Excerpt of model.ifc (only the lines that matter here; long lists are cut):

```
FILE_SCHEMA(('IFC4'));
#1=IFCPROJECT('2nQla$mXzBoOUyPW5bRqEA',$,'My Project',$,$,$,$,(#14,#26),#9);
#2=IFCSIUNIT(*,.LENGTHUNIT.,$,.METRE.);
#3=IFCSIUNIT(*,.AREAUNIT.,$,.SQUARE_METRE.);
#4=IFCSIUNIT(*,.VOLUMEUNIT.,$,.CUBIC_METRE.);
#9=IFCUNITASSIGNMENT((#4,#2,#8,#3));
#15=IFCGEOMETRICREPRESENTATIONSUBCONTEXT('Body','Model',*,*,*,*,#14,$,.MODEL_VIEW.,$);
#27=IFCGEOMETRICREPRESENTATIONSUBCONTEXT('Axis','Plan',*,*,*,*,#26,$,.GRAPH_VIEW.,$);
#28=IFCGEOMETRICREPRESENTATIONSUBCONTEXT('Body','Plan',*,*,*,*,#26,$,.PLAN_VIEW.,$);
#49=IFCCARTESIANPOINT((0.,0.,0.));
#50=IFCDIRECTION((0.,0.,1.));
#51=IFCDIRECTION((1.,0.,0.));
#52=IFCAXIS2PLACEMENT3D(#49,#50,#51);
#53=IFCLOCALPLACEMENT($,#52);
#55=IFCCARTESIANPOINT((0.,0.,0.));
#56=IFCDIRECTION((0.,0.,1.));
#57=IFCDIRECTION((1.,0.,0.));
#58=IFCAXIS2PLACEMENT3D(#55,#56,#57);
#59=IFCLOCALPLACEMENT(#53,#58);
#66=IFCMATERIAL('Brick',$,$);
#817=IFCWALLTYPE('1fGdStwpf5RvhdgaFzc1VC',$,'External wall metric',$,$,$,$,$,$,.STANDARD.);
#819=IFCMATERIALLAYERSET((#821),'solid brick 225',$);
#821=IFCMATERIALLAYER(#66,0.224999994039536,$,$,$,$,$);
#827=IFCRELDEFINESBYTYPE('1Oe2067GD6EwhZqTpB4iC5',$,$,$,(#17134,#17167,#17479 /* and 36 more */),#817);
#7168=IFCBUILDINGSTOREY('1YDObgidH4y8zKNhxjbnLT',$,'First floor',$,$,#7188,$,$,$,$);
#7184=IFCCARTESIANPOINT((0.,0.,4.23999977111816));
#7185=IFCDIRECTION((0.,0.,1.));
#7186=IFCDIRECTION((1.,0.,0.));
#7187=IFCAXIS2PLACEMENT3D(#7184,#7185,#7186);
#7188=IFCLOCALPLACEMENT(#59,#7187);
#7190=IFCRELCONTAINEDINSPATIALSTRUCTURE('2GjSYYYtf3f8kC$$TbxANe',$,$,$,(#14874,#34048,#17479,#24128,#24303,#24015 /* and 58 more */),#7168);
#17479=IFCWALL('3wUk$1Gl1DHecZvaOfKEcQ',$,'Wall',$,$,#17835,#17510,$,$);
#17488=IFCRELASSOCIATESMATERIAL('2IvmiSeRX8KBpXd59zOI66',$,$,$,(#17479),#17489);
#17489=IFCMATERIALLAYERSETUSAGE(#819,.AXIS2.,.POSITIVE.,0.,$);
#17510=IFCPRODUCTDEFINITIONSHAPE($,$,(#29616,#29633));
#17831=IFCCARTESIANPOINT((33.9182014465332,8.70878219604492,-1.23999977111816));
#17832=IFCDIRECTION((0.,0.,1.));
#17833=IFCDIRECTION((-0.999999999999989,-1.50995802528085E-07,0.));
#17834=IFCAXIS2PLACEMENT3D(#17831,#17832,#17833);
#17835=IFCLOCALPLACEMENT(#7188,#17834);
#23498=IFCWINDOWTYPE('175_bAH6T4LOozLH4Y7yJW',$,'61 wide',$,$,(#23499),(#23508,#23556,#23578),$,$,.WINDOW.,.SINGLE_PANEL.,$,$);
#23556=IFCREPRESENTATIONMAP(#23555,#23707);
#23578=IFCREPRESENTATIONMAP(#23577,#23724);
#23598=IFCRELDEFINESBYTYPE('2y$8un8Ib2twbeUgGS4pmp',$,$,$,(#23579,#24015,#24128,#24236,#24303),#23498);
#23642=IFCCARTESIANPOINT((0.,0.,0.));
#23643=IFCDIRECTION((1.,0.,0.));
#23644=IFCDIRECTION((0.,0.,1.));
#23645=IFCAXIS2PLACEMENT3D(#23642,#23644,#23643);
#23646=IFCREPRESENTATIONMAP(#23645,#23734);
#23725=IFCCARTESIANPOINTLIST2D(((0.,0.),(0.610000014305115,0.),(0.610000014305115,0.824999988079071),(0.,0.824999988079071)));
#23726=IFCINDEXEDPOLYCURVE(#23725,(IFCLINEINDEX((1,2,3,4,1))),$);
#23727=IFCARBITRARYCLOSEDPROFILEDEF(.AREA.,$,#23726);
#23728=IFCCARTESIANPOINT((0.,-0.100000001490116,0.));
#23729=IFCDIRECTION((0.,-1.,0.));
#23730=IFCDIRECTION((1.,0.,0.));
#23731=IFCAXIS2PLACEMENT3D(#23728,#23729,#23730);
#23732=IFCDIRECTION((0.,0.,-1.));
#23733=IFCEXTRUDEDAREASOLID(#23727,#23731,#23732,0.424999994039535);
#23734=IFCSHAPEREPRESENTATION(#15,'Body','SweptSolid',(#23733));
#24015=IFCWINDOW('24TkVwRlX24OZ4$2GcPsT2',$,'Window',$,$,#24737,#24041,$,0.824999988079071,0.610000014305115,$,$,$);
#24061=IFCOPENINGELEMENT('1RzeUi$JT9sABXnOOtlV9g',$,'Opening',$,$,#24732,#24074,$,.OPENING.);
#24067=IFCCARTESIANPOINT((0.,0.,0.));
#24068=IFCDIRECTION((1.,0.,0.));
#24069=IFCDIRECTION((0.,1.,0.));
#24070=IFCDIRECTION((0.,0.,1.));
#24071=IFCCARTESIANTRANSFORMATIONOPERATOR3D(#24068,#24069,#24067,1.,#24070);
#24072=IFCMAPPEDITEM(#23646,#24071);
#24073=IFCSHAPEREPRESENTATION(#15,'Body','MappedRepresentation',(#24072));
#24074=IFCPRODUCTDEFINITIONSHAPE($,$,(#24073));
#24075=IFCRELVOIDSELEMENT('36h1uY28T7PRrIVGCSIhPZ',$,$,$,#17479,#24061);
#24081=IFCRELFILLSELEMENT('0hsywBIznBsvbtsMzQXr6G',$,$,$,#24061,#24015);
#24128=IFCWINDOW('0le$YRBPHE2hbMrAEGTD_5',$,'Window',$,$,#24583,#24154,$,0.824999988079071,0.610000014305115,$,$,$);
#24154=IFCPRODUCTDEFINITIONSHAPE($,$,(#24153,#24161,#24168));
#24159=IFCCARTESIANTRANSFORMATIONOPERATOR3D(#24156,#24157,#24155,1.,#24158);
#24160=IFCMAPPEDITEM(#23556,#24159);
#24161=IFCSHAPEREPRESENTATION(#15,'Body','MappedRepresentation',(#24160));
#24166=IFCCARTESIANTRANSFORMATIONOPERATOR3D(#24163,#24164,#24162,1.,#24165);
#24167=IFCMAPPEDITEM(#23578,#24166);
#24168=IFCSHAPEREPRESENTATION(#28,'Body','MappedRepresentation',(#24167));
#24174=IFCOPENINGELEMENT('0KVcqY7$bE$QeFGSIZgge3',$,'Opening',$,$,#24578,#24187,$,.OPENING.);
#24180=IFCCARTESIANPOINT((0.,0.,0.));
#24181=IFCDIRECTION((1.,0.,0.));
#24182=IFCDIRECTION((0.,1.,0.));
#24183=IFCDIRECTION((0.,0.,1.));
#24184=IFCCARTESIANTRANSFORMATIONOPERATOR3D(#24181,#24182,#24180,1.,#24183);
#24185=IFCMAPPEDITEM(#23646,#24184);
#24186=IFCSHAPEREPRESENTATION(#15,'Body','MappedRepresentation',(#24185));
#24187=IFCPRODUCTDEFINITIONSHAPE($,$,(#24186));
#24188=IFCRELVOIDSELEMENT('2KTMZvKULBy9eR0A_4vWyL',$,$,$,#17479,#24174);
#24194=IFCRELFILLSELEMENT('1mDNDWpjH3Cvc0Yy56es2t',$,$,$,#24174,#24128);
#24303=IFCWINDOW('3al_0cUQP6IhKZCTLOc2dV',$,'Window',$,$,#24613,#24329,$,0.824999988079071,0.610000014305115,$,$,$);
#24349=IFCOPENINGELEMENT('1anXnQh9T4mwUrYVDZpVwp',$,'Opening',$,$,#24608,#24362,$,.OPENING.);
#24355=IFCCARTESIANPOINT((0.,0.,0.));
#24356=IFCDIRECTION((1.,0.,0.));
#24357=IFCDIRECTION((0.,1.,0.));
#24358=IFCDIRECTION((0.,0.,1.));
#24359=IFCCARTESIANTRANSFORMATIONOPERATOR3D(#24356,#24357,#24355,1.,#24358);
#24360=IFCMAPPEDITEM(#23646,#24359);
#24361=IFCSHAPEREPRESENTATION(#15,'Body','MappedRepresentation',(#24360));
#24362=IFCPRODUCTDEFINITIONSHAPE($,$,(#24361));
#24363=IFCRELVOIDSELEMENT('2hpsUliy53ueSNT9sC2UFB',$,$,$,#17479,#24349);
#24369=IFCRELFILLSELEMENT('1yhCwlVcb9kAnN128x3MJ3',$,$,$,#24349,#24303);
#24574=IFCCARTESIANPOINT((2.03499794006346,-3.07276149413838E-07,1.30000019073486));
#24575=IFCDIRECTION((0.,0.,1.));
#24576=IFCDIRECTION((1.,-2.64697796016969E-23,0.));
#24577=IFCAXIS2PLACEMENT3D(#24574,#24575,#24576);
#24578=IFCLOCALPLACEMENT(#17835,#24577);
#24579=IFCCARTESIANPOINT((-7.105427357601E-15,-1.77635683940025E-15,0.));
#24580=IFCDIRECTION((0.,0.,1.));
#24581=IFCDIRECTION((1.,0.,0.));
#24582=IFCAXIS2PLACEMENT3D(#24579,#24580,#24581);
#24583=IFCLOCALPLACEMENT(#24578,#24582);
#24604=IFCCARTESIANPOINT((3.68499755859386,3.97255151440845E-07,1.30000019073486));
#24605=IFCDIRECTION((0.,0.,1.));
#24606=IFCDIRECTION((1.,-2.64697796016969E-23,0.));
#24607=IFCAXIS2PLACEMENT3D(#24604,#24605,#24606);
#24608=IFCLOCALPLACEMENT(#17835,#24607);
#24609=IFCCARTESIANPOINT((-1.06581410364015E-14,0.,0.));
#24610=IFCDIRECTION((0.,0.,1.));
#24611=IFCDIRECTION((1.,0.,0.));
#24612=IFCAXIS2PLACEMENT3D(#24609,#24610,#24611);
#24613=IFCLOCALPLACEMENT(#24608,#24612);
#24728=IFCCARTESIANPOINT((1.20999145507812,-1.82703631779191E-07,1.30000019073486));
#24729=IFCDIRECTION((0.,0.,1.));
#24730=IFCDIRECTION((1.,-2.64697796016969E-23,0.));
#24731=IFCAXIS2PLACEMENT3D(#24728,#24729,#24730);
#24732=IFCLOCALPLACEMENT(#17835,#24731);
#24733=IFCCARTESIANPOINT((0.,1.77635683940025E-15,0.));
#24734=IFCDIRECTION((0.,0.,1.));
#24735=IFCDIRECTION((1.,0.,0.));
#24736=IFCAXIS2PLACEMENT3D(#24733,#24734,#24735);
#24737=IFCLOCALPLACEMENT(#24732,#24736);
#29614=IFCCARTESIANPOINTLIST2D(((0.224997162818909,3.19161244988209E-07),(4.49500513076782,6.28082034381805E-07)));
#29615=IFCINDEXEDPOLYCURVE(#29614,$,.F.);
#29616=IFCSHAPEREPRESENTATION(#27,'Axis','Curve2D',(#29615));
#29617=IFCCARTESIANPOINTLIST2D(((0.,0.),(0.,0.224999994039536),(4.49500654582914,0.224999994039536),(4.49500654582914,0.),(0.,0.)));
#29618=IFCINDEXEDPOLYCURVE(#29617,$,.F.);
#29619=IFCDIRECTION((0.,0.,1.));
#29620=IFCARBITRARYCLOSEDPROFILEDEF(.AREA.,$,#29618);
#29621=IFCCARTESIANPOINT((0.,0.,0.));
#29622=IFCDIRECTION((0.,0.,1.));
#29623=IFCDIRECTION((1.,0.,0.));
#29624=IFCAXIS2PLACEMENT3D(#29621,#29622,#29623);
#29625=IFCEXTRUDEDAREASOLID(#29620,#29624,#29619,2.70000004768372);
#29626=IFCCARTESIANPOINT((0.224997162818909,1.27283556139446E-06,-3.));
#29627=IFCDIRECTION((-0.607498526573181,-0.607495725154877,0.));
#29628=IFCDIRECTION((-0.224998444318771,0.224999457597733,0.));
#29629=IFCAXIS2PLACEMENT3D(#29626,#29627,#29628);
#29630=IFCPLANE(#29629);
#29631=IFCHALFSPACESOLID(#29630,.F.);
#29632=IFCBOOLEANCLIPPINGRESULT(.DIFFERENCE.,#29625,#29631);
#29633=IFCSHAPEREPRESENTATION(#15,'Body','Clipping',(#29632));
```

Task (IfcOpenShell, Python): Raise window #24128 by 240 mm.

```python
import numpy as np
import ifcopenshell
import ifcopenshell.api.geometry
import ifcopenshell.util.placement
import ifcopenshell.util.unit

model = ifcopenshell.open("model.ifc")
unit_scale = ifcopenshell.util.unit.calculate_unit_scale(model)

window = model.by_guid("0le$YRBPHE2hbMrAEGTD_5")
opening = window.FillsVoids[0].RelatingOpeningElement
dz = 0.24

shift = np.array([0.0, 0.0, dz])
# The window is placed relative to its opening, so it follows when the opening moves.
matrix = ifcopenshell.util.placement.get_local_placement(opening.ObjectPlacement)
matrix[:3, 3] += shift
ifcopenshell.api.geometry.edit_object_placement(
    model, product=opening, matrix=matrix, is_si=False, should_transform_children=True
)

print(f"moved by {dz * unit_scale:+.3f} m")

model.write("model_rev.ifc")
```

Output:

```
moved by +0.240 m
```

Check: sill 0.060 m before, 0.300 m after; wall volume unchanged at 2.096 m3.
